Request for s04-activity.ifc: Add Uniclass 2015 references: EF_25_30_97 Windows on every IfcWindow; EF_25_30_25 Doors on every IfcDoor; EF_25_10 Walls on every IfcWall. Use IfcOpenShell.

First a look at what the model holds.

```python
import ifcopenshell

model = ifcopenshell.open("s04-activity.ifc")
print(model.schema)
print("classifications:", [c.Name for c in model.by_type("IfcClassification")])
for ifc_class in ("IfcDoor", "IfcRoof", "IfcStair", "IfcWall", "IfcWindow"):
    print(ifc_class, len(model.by_type(ifc_class)))
```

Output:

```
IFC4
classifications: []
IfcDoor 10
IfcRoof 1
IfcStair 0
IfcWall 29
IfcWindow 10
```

```python
import ifcopenshell
import ifcopenshell.api.classification

model = ifcopenshell.open("s04-activity.ifc")

system = ifcopenshell.api.classification.add_classification(model, classification="Uniclass 2015")

codes = {
    "IfcWindow": ("EF_25_30_97", "Windows"),
    "IfcDoor": ("EF_25_30_25", "Doors"),
    "IfcWall": ("EF_25_10", "Walls"),
}
for ifc_class, (code, name) in codes.items():
    products = model.by_type(ifc_class)
    ifcopenshell.api.classification.add_reference(
        model, products=products, classification=system, identification=code, name=name
    )
    print(code, len(products))

model.write("s04-activity_updated.ifc")
```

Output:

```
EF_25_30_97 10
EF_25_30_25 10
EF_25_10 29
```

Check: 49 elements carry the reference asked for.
